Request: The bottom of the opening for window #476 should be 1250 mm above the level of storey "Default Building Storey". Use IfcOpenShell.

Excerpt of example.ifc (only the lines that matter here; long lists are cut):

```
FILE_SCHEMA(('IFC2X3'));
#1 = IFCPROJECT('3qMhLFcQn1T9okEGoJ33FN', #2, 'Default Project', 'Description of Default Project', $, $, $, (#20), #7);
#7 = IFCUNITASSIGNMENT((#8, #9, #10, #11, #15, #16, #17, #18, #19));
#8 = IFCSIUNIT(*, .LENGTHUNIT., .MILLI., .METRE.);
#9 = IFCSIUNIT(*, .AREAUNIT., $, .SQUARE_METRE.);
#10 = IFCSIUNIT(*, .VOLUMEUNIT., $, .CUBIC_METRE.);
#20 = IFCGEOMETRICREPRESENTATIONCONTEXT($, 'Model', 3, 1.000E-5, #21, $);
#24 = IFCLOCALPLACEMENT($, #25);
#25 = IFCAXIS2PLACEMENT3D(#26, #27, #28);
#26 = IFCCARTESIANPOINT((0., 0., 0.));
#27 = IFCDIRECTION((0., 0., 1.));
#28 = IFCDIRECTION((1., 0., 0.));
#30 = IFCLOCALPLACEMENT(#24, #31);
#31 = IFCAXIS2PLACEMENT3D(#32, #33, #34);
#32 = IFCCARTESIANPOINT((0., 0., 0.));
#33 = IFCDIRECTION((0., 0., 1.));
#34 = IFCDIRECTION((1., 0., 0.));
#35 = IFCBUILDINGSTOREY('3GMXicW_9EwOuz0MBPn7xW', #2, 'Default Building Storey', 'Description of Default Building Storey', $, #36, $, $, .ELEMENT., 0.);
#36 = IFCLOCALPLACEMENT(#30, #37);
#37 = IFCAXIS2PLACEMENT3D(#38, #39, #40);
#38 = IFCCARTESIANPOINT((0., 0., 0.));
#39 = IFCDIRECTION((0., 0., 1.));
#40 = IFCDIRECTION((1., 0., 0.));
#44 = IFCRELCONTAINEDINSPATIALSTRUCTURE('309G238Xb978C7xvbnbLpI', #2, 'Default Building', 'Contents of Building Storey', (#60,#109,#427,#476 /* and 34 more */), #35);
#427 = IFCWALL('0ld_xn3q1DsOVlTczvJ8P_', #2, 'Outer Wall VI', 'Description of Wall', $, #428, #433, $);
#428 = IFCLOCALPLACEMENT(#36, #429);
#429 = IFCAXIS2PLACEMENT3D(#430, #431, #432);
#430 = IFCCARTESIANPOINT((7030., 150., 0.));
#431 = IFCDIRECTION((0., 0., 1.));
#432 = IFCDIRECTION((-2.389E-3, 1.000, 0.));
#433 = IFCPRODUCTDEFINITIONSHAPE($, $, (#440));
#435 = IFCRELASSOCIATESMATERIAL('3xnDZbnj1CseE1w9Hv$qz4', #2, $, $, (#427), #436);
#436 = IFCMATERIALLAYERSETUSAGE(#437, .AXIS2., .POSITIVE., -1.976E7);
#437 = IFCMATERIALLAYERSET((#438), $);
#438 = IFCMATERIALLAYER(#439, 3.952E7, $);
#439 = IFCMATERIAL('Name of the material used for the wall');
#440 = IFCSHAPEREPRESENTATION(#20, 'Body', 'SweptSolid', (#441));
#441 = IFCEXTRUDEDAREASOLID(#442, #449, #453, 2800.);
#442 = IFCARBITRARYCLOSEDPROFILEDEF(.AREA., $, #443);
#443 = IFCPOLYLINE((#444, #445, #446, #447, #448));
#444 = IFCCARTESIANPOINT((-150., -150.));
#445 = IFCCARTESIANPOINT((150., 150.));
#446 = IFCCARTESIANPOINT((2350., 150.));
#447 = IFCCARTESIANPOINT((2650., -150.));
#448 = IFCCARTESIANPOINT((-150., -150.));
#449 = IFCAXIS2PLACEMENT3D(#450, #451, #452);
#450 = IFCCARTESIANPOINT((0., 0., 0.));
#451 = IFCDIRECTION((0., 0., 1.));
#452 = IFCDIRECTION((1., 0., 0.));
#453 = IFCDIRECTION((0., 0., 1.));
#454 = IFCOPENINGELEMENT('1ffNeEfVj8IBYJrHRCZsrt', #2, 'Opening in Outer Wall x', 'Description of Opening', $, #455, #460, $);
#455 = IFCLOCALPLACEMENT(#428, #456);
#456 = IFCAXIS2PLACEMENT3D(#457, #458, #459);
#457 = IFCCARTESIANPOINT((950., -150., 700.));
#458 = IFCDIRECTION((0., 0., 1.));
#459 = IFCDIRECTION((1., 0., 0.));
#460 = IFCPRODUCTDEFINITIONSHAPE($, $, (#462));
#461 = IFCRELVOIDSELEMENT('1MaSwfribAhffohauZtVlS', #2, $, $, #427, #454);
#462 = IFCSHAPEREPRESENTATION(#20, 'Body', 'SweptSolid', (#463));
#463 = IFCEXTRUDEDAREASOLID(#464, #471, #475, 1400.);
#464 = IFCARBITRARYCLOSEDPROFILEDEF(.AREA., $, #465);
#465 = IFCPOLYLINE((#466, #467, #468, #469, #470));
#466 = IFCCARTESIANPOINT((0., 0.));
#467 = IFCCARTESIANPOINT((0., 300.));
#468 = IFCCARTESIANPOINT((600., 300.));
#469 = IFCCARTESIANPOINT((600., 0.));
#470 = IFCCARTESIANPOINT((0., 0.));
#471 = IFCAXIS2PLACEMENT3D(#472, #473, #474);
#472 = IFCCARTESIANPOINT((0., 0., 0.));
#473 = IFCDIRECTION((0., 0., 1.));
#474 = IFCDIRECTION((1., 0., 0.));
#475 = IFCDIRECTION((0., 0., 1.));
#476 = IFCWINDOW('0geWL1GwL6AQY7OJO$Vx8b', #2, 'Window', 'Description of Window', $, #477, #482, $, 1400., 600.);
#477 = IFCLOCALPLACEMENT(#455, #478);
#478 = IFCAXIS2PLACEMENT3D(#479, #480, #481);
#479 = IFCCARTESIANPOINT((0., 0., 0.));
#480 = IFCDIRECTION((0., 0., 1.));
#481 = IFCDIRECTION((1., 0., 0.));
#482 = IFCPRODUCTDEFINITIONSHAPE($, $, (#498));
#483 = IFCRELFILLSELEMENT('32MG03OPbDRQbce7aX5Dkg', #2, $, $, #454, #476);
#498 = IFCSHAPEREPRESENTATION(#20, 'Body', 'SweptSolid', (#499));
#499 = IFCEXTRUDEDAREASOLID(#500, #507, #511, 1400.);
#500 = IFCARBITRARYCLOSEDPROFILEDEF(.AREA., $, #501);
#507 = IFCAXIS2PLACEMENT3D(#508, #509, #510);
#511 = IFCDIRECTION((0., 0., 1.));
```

```python
import numpy as np
import ifcopenshell
import ifcopenshell.api.geometry
import ifcopenshell.geom
import ifcopenshell.util.element
import ifcopenshell.util.placement
import ifcopenshell.util.shape
import ifcopenshell.util.unit

model = ifcopenshell.open("example.ifc")
unit_scale = ifcopenshell.util.unit.calculate_unit_scale(model)

window = model.by_guid("0geWL1GwL6AQY7OJO$Vx8b")
opening = window.FillsVoids[0].RelatingOpeningElement
storey = ifcopenshell.util.element.get_container(window, ifc_class="IfcBuildingStorey")
level = ifcopenshell.util.placement.get_local_placement(storey.ObjectPlacement)[2, 3]

# The opening's origin need not be at the sill, so measure its lowest point.
shape = ifcopenshell.geom.create_shape(ifcopenshell.geom.settings(), opening)
bottom = ifcopenshell.util.shape.get_shape_bottom_elevation(shape, shape.geometry) / unit_scale
dz = level + 1.25 / unit_scale - bottom

shift = np.array([0.0, 0.0, dz])
# The window is placed relative to its opening, so it follows when the opening moves.
matrix = ifcopenshell.util.placement.get_local_placement(opening.ObjectPlacement)
matrix[:3, 3] += shift
ifcopenshell.api.geometry.edit_object_placement(
    model, product=opening, matrix=matrix, is_si=False, should_transform_children=True
)

print(f"moved by {dz * unit_scale:+.3f} m")

model.write("example_edited.ifc")
```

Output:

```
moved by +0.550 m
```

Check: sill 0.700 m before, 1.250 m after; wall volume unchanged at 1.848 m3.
